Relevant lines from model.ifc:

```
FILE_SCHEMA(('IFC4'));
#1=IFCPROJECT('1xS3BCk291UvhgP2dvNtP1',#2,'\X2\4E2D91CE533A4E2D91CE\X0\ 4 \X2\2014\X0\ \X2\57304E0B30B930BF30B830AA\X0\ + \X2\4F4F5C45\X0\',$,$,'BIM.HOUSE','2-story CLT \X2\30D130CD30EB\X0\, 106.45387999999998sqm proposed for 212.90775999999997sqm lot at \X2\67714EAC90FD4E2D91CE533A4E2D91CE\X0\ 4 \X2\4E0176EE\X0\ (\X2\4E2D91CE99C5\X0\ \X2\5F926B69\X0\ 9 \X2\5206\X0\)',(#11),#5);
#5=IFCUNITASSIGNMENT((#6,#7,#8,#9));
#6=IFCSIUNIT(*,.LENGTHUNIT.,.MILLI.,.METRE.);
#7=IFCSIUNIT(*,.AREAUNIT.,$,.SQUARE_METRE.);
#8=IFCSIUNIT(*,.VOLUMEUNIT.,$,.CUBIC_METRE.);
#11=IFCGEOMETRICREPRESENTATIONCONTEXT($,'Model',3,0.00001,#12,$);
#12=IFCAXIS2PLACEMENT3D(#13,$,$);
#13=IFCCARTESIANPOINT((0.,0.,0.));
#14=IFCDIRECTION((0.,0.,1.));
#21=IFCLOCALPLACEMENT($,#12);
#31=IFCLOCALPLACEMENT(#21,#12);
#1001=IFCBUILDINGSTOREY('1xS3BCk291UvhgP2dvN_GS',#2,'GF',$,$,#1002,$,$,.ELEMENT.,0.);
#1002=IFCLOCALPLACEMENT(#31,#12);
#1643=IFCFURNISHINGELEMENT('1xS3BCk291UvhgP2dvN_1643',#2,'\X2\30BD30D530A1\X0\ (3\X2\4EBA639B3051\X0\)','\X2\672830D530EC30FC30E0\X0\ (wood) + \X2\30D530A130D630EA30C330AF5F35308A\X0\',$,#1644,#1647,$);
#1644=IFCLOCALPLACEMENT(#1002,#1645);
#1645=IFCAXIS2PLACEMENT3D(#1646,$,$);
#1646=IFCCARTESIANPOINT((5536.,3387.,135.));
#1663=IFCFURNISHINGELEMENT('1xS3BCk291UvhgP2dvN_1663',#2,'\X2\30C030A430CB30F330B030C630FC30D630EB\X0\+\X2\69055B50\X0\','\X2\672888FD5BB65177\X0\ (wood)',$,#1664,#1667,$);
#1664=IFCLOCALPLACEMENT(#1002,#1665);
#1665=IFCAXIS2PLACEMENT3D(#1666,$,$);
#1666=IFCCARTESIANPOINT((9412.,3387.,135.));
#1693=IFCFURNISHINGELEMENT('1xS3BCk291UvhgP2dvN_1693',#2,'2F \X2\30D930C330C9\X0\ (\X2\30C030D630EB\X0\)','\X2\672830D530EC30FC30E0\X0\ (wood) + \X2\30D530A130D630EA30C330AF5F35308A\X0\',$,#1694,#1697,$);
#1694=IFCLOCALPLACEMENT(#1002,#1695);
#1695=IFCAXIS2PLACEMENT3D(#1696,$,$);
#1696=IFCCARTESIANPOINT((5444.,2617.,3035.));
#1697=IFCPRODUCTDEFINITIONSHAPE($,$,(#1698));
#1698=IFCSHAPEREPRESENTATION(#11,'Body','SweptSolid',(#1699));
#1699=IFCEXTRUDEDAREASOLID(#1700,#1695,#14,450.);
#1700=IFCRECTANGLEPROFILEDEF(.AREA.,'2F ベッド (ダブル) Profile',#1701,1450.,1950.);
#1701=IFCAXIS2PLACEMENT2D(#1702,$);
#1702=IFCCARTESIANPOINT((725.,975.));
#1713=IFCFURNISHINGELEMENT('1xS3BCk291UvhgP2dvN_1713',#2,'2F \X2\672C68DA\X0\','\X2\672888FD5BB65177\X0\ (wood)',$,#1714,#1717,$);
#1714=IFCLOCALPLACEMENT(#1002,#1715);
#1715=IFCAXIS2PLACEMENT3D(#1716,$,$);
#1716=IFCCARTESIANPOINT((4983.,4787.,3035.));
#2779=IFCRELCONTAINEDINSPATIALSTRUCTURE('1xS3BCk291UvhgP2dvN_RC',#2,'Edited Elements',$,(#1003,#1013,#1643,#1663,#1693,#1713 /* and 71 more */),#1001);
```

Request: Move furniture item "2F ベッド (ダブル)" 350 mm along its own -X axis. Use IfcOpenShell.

```python
import ifcopenshell
import ifcopenshell.api.geometry
import ifcopenshell.util.placement
import ifcopenshell.util.unit

model = ifcopenshell.open("model.ifc")
unit_scale = ifcopenshell.util.unit.calculate_unit_scale(model)

item = model.by_id(1693)
matrix = ifcopenshell.util.placement.get_local_placement(item.ObjectPlacement)
matrix[:3, 3] -= matrix[:3, 0] * 0.35 / unit_scale
ifcopenshell.api.geometry.edit_object_placement(model, product=item, matrix=matrix, is_si=False)

print(ifcopenshell.util.placement.get_local_placement(item.ObjectPlacement).round(3) + 0.0)

model.write("model_v2.ifc")
```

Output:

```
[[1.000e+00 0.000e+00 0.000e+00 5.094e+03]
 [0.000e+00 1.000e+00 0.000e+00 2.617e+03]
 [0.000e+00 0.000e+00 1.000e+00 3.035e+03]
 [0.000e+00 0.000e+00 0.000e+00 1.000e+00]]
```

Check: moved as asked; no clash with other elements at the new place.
